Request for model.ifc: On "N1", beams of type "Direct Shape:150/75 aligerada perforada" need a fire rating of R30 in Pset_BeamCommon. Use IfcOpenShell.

First a look at what the model holds.

```python
import ifcopenshell
import ifcopenshell.util.element

model = ifcopenshell.open("model.ifc")
print(model.schema)
storey = next(s for s in model.by_type("IfcBuildingStorey") if s.Name == "N1")
beams = [e for e in ifcopenshell.util.element.get_decomposition(storey) if e.is_a("IfcBeam")]
seen = {}
for e in beams:
    element_type = ifcopenshell.util.element.get_type(e)
    key = (element_type.Name if element_type != e and element_type else None, ifcopenshell.util.element.get_pset(e, "Pset_BeamCommon", "FireRating"))
    seen[key] = seen.get(key, 0) + 1
for (name, value), count in sorted(seen.items(), key=str):
    print(count, "x", name, "|", value)
```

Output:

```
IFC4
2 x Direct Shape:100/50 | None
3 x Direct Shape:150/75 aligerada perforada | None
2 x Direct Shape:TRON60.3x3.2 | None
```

```python
import ifcopenshell
import ifcopenshell.api.pset
import ifcopenshell.util.element

model = ifcopenshell.open("model.ifc")

storey = next(s for s in model.by_type("IfcBuildingStorey") if s.Name == "N1")
beams = [e for e in ifcopenshell.util.element.get_decomposition(storey) if e.is_a("IfcBeam")]

count = 0
for e in beams:
    element_type = ifcopenshell.util.element.get_type(e)
    if element_type in (None, e) or element_type.Name != "Direct Shape:150/75 aligerada perforada":
        continue
    # add_pset returns the element's existing set when there is one.
    pset = ifcopenshell.api.pset.add_pset(model, product=e, name="Pset_BeamCommon")
    ifcopenshell.api.pset.edit_pset(model, pset=pset, properties={"FireRating": "R30"})
    count += 1

print(count, "beams updated")

model.write("model_edited.ifc")
```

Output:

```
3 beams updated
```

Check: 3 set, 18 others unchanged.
